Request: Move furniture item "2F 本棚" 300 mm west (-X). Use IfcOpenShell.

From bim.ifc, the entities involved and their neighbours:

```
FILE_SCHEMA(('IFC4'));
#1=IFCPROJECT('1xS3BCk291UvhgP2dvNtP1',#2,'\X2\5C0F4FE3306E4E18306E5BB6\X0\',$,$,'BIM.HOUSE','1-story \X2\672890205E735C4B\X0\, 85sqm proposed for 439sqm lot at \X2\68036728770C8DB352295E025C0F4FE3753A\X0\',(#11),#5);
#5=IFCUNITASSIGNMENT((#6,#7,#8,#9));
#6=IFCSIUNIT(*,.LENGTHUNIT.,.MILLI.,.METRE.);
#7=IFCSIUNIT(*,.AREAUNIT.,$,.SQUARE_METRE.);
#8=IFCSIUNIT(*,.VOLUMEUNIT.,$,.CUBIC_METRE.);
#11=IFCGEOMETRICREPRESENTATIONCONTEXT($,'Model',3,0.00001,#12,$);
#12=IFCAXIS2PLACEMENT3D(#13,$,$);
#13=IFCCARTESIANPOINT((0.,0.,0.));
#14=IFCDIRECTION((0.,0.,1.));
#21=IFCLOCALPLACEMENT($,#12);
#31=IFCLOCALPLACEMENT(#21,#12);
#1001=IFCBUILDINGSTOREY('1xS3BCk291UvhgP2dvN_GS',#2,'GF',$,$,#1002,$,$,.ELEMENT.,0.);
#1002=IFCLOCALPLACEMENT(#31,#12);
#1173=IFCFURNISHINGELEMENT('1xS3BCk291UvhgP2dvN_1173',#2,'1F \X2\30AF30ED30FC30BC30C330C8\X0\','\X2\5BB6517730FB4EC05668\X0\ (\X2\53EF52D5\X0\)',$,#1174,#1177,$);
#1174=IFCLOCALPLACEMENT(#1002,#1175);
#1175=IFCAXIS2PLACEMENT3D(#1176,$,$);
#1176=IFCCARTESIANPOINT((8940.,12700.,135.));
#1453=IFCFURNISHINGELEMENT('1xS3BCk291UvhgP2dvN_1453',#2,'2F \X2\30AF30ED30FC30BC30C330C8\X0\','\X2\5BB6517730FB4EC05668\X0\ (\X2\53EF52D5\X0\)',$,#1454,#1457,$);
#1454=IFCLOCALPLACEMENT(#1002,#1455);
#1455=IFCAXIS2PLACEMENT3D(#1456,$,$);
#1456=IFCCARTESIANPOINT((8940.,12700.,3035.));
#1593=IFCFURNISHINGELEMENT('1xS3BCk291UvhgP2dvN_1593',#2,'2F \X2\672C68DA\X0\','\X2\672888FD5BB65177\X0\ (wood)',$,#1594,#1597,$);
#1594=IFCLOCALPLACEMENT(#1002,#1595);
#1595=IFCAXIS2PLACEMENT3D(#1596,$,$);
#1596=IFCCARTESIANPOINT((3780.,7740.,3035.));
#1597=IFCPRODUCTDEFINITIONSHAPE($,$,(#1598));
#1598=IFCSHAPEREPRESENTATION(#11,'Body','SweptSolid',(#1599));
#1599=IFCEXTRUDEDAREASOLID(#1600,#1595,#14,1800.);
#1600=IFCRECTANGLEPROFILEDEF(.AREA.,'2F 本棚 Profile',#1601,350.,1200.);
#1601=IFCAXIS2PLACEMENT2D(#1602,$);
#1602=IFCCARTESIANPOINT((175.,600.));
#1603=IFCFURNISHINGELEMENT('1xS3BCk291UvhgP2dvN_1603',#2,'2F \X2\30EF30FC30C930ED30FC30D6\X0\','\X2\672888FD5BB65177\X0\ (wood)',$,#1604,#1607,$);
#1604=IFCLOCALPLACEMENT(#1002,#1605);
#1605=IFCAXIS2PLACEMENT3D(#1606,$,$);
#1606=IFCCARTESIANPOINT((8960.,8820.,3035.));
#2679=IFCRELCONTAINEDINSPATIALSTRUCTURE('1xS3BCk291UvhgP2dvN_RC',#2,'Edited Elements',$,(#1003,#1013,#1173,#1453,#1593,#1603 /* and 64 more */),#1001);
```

```python
import ifcopenshell
import ifcopenshell.api.geometry
import ifcopenshell.util.placement

model = ifcopenshell.open("bim.ifc")

item = model.by_guid("1xS3BCk291UvhgP2dvN_1593")
matrix = ifcopenshell.util.placement.get_local_placement(item.ObjectPlacement)
matrix[0, 3] -= 300.0
ifcopenshell.api.geometry.edit_object_placement(model, product=item, matrix=matrix, is_si=False)

print(ifcopenshell.util.placement.get_local_placement(item.ObjectPlacement).round(3) + 0.0)

model.write("bim_updated.ifc")
```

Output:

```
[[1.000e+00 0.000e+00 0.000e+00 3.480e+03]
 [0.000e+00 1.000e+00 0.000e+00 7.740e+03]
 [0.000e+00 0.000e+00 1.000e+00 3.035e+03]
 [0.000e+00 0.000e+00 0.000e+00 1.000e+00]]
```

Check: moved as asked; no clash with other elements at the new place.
